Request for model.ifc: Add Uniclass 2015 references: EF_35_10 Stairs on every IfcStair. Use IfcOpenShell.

First a look at what the model holds.

```python
import ifcopenshell

model = ifcopenshell.open("model.ifc")
print(model.schema)
print("classifications:", [c.Name for c in model.by_type("IfcClassification")])
for ifc_class in ("IfcDoor", "IfcRoof", "IfcStair", "IfcWall", "IfcWindow"):
    print(ifc_class, len(model.by_type(ifc_class)))
```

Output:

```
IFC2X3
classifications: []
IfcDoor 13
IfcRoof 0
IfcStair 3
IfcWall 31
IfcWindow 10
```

```python
import ifcopenshell
import ifcopenshell.api.classification

model = ifcopenshell.open("model.ifc")

# IFC2X3 requires Source and Edition and has no link from the project to the system.
system = model.create_entity("IfcClassification", Source="NBS", Edition="2015", Name="Uniclass 2015")

codes = {
    "IfcStair": ("EF_35_10", "Stairs"),
}
for ifc_class, (code, name) in codes.items():
    products = model.by_type(ifc_class)
    ifcopenshell.api.classification.add_reference(
        model, products=products, classification=system, identification=code, name=name
    )
    print(code, len(products))

model.write("model_updated.ifc")
```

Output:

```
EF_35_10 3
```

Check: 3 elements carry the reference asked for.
